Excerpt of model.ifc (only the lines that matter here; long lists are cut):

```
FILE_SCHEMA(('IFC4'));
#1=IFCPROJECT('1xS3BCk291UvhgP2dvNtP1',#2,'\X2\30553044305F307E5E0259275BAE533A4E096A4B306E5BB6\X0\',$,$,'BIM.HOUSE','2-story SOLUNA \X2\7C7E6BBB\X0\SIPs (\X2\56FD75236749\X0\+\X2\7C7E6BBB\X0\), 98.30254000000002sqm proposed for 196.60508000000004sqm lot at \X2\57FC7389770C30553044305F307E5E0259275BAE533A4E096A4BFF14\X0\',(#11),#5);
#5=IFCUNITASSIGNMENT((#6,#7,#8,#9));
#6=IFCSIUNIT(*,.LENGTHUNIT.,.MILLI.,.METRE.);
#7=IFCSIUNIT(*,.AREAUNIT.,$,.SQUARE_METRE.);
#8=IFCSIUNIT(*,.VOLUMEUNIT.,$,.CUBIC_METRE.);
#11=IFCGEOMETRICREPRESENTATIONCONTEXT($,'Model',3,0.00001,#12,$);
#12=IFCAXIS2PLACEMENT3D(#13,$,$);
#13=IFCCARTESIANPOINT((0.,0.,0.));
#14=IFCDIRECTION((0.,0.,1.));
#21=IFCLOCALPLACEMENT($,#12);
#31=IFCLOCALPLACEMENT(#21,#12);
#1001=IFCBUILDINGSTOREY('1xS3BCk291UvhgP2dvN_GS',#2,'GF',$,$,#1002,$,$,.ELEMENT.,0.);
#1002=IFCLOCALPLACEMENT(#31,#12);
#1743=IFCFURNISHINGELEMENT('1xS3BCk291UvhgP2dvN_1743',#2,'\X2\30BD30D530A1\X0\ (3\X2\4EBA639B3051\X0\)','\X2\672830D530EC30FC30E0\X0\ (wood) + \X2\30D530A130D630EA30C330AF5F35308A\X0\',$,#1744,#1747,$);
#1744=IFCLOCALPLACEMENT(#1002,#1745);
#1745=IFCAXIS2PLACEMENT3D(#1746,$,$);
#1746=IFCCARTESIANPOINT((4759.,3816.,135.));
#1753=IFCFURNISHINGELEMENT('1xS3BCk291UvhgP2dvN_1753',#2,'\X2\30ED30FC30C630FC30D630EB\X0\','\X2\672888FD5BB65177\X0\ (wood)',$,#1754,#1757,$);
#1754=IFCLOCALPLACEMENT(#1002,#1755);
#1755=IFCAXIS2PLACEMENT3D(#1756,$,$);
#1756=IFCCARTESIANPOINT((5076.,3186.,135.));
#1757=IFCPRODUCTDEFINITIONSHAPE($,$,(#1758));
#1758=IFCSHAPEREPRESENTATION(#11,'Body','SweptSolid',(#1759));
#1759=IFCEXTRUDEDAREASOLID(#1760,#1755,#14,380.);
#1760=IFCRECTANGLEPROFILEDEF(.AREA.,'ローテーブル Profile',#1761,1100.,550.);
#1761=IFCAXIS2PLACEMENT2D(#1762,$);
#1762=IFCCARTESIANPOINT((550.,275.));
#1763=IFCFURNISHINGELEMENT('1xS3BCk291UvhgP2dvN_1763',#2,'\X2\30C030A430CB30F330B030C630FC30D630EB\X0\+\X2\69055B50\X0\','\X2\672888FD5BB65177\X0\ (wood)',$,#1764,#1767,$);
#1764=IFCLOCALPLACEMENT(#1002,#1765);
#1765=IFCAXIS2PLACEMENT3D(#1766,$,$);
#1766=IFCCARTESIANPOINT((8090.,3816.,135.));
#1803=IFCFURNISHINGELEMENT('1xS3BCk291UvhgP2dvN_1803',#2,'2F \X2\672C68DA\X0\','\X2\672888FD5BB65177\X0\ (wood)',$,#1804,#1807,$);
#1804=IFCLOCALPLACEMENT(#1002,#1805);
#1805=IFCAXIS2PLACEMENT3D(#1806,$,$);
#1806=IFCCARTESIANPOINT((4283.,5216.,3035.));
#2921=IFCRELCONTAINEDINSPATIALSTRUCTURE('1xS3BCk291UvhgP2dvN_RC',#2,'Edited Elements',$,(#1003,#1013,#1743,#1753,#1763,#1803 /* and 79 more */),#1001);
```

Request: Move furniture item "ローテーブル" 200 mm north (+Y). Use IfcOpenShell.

```python
import ifcopenshell
import ifcopenshell.api.geometry
import ifcopenshell.util.placement
import ifcopenshell.util.unit

model = ifcopenshell.open("model.ifc")
unit_scale = ifcopenshell.util.unit.calculate_unit_scale(model)

item = model.by_guid("1xS3BCk291UvhgP2dvN_1753")
matrix = ifcopenshell.util.placement.get_local_placement(item.ObjectPlacement)
matrix[1, 3] += 0.2 / unit_scale
ifcopenshell.api.geometry.edit_object_placement(model, product=item, matrix=matrix, is_si=False)

print(ifcopenshell.util.placement.get_local_placement(item.ObjectPlacement).round(3) + 0.0)

model.write("model_updated.ifc")
```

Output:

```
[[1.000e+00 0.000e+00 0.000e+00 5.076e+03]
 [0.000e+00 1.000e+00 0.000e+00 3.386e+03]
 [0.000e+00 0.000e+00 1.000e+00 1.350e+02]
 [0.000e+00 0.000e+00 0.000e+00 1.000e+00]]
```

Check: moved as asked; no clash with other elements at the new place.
